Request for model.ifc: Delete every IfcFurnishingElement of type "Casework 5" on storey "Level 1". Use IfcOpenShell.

First a look at what the model holds.

```python
import ifcopenshell
import ifcopenshell.util.element

model = ifcopenshell.open("model.ifc")
print(model.schema)
storey = next(s for s in model.by_type("IfcBuildingStorey") if s.Name == "Level 1")
furniture = [e for e in ifcopenshell.util.element.get_decomposition(storey) if e.is_a("IfcFurnishingElement")]
seen = {}
for e in furniture:
    element_type = ifcopenshell.util.element.get_type(e)
    name = element_type.Name if element_type not in (None, e) else None
    seen[name] = seen.get(name, 0) + 1
for name, count in sorted(seen.items(), key=str):
    print(count, "x", name)
```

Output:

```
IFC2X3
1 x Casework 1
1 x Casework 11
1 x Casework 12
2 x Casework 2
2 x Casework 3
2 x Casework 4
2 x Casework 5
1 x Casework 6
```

```python
import ifcopenshell
import ifcopenshell.api.root
import ifcopenshell.util.element

model = ifcopenshell.open("model.ifc")

storey = next(s for s in model.by_type("IfcBuildingStorey") if s.Name == "Level 1")
furniture = [e for e in ifcopenshell.util.element.get_decomposition(storey) if e.is_a("IfcFurnishingElement")]
targets = [e for e in furniture if (t := ifcopenshell.util.element.get_type(e)) not in (None, e) and t.Name == "Casework 5"]

for e in targets:
    ifcopenshell.api.root.remove_product(model, product=e)
print(len(targets), "removed")

model.write("model_rev.ifc")
```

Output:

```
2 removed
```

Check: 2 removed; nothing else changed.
